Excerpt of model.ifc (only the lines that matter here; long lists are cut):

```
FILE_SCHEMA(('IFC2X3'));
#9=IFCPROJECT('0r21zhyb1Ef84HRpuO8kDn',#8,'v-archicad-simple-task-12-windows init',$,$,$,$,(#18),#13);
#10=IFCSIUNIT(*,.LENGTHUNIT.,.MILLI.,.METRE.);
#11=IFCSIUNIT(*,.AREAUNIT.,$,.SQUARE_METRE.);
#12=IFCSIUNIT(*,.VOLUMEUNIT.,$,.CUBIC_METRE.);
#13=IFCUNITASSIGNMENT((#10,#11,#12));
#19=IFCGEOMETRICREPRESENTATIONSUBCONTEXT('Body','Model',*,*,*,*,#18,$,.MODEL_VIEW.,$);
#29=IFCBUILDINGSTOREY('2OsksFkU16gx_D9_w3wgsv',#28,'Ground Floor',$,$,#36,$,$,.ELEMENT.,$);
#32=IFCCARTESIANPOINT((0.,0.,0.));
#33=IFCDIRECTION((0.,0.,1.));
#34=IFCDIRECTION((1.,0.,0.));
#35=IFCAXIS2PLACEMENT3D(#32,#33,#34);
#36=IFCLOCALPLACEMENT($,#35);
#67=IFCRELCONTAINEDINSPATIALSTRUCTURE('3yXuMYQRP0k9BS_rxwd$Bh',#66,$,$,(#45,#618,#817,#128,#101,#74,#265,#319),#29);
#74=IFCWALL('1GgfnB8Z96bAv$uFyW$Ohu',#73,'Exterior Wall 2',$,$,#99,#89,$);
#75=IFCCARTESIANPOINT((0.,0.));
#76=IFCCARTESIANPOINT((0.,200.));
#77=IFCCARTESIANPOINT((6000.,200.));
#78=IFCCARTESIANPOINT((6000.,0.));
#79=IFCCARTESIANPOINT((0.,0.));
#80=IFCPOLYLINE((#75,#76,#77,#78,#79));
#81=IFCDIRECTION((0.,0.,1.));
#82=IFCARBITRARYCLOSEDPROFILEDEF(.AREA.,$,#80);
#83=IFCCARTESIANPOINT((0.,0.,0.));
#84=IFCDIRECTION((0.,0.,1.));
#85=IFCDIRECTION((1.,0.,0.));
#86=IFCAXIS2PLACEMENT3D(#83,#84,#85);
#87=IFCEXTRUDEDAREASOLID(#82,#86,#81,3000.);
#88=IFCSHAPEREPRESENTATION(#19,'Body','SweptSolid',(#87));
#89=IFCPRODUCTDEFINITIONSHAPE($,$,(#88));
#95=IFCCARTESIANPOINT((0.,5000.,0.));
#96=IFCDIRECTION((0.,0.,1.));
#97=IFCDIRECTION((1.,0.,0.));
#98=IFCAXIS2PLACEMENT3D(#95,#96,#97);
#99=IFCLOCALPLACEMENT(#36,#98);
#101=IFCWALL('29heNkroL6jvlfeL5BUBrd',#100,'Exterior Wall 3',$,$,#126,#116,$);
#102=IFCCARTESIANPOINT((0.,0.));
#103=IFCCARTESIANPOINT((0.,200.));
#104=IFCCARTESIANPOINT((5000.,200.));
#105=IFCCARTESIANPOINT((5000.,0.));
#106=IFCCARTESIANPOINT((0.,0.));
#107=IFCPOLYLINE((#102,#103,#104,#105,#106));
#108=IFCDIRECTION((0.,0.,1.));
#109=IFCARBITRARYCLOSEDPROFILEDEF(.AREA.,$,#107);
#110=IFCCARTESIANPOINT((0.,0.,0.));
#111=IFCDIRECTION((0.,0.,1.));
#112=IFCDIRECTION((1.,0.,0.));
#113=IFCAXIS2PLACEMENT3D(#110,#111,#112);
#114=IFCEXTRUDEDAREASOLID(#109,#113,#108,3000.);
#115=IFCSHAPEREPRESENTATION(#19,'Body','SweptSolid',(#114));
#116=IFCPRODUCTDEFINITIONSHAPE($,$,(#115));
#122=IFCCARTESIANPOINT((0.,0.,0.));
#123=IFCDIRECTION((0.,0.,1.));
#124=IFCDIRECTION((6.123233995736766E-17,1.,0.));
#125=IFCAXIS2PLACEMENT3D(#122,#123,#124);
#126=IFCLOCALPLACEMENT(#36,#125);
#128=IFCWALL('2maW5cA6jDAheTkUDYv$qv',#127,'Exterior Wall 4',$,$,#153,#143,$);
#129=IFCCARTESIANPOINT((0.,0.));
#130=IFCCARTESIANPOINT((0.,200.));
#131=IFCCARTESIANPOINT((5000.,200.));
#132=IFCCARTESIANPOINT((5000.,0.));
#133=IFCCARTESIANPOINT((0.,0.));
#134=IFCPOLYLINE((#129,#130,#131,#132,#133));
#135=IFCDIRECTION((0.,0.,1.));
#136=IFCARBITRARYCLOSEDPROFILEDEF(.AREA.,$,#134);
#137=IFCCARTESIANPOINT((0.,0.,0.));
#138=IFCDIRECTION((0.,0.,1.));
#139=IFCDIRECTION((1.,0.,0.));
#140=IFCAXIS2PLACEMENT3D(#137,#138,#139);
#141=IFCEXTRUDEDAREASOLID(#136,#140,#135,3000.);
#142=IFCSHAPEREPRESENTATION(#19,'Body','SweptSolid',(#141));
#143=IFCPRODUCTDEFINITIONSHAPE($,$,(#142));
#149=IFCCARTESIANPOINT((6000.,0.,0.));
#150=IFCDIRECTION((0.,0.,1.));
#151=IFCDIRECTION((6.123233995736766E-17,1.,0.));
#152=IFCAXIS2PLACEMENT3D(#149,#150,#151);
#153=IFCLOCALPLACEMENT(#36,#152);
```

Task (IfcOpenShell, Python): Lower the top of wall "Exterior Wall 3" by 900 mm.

```python
import ifcopenshell
import ifcopenshell.geom
import ifcopenshell.util.representation
import ifcopenshell.util.shape
import ifcopenshell.util.unit

model = ifcopenshell.open("model.ifc")
unit_scale = ifcopenshell.util.unit.calculate_unit_scale(model)
settings = ifcopenshell.geom.settings()


def volume(element):
    """Net volume in cubic metres, openings subtracted."""
    shape = ifcopenshell.geom.create_shape(settings, element)
    return ifcopenshell.util.shape.get_volume(shape.geometry)


wall = model.by_guid("29heNkroL6jvlfeL5BUBrd")
before = volume(wall)

body = ifcopenshell.util.representation.get_representation(wall, "Model", "Body")
solid = body.Items[0]
old_height = solid.Depth
solid.Depth -= 0.9 / unit_scale
after = volume(wall)

print(f"height {old_height:g} -> {solid.Depth:g}, volume {before:.3f} -> {after:.3f} m3")

model.write("model_v2.ifc")
```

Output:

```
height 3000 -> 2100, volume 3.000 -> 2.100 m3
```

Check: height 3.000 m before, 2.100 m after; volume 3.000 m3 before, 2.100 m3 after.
